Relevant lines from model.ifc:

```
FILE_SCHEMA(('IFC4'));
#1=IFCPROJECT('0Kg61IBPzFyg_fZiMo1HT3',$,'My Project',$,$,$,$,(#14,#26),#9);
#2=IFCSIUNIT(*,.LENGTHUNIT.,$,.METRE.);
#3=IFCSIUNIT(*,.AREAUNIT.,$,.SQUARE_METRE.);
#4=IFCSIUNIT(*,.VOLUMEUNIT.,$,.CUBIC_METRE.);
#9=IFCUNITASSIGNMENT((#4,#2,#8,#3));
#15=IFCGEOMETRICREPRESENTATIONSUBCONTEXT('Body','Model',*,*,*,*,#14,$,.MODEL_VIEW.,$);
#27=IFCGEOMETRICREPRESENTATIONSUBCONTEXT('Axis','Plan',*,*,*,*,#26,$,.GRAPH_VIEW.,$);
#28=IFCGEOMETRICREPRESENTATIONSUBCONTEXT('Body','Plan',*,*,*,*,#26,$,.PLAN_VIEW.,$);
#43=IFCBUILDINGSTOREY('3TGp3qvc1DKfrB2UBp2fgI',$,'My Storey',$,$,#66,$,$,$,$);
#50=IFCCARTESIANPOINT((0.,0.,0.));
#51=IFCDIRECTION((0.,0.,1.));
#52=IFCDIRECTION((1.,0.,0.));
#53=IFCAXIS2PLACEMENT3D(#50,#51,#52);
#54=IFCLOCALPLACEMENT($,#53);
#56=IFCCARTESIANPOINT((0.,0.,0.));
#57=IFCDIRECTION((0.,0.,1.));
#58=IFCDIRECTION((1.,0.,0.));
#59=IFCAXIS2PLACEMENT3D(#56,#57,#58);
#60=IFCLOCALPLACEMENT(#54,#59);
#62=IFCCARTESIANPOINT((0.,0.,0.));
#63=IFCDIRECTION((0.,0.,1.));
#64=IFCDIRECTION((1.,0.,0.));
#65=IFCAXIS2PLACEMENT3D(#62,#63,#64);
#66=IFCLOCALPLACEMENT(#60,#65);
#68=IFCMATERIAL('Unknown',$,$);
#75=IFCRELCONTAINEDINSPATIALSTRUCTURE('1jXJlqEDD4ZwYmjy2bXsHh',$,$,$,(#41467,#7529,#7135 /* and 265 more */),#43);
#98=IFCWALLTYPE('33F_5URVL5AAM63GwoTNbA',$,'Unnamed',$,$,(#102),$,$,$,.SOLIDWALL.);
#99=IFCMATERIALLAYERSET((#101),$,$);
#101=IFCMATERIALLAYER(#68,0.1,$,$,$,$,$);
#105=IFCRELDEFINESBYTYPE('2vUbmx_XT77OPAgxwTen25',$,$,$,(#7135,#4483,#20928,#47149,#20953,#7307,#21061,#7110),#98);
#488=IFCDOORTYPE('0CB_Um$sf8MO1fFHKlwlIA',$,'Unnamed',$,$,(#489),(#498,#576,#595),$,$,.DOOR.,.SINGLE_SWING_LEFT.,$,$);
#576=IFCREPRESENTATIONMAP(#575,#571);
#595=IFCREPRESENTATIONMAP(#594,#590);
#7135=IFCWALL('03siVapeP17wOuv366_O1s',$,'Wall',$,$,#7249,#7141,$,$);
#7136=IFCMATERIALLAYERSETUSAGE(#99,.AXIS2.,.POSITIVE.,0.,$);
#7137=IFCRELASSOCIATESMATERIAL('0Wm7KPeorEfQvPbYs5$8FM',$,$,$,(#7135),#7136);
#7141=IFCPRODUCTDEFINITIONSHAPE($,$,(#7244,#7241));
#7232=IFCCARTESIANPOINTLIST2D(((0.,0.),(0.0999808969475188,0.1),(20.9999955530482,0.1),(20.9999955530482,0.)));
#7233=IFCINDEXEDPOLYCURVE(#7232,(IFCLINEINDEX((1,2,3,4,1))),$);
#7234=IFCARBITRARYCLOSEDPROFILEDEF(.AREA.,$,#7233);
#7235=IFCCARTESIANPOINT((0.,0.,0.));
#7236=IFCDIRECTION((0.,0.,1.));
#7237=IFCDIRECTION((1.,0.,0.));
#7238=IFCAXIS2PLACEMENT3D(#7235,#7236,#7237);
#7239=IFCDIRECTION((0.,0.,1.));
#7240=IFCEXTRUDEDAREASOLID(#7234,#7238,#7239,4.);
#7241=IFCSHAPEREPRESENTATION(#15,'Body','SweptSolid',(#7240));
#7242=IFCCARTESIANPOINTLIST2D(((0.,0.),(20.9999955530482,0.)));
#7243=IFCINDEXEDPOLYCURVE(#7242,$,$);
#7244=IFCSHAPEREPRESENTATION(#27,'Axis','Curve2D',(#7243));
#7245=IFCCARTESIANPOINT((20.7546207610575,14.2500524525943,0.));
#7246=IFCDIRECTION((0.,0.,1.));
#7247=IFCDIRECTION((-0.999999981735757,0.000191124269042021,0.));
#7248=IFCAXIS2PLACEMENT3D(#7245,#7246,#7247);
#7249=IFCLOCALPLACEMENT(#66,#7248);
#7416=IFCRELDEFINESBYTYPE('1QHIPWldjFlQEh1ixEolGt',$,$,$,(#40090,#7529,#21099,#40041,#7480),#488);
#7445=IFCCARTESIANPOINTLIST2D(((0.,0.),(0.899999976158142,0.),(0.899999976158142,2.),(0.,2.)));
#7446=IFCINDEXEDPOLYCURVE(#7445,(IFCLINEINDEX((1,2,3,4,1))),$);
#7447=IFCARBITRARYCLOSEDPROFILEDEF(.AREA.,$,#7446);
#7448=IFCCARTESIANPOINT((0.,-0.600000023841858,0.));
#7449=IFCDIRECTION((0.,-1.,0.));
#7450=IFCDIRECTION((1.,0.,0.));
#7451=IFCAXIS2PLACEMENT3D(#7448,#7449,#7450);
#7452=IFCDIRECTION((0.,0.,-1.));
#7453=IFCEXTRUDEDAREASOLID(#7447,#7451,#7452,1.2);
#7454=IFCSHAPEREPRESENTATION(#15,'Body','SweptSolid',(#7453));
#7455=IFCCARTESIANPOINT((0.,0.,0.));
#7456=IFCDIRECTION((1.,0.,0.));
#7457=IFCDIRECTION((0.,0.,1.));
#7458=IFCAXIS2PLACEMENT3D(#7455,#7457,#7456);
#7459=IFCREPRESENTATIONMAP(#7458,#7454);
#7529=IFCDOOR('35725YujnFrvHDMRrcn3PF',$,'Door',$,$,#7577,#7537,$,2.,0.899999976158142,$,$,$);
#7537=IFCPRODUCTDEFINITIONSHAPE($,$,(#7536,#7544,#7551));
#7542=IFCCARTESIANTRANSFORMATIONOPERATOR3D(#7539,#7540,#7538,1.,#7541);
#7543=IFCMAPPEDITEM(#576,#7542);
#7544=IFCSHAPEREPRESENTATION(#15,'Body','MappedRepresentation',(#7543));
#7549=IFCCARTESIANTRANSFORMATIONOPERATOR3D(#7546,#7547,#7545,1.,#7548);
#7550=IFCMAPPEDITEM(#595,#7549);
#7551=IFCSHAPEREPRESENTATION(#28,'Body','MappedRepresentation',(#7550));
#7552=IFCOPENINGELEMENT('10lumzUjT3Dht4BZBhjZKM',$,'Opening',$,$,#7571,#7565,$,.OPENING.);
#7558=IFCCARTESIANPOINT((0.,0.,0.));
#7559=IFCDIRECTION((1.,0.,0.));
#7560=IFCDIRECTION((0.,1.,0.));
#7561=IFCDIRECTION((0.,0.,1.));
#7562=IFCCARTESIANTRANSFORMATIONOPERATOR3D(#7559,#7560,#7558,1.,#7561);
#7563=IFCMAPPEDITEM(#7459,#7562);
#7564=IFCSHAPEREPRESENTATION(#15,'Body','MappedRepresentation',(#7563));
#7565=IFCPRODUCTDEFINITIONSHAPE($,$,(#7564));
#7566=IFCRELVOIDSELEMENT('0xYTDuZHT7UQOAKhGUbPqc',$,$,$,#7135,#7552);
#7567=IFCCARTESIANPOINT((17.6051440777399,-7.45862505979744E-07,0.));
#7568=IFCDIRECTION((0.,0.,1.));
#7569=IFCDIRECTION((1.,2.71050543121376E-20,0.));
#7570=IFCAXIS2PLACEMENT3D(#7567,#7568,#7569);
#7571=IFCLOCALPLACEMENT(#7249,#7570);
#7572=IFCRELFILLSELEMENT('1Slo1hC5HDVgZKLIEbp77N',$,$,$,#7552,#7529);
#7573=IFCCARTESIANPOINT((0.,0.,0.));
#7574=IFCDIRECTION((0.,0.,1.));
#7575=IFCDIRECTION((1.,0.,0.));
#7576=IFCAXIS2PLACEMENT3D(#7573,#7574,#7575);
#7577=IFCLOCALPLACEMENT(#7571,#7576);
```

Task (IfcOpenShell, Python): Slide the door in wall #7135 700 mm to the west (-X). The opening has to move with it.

```python
import ifcopenshell
import ifcopenshell.api.geometry
import ifcopenshell.util.placement

model = ifcopenshell.open("model.ifc")

door = model.by_guid("35725YujnFrvHDMRrcn3PF")
opening = door.FillsVoids[0].RelatingOpeningElement
wall = opening.VoidsElements[0].RelatingBuildingElement

wall_matrix = ifcopenshell.util.placement.get_local_placement(wall.ObjectPlacement)
shift = wall_matrix[:3, 0] * 0.7
before = ifcopenshell.util.placement.get_local_placement(door.ObjectPlacement)[:3, 3].copy()

# The door is placed relative to its opening, so it follows when the opening moves.
matrix = ifcopenshell.util.placement.get_local_placement(opening.ObjectPlacement)
matrix[:3, 3] += shift
ifcopenshell.api.geometry.edit_object_placement(
    model, product=opening, matrix=matrix, is_si=False, should_transform_children=True
)

after = ifcopenshell.util.placement.get_local_placement(door.ObjectPlacement)[:3, 3]
print("door moved by", (after - before).round(3) + 0.0)

model.write("model_v2.ifc")
```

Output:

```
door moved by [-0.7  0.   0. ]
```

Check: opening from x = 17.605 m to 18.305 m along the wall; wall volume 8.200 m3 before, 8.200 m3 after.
